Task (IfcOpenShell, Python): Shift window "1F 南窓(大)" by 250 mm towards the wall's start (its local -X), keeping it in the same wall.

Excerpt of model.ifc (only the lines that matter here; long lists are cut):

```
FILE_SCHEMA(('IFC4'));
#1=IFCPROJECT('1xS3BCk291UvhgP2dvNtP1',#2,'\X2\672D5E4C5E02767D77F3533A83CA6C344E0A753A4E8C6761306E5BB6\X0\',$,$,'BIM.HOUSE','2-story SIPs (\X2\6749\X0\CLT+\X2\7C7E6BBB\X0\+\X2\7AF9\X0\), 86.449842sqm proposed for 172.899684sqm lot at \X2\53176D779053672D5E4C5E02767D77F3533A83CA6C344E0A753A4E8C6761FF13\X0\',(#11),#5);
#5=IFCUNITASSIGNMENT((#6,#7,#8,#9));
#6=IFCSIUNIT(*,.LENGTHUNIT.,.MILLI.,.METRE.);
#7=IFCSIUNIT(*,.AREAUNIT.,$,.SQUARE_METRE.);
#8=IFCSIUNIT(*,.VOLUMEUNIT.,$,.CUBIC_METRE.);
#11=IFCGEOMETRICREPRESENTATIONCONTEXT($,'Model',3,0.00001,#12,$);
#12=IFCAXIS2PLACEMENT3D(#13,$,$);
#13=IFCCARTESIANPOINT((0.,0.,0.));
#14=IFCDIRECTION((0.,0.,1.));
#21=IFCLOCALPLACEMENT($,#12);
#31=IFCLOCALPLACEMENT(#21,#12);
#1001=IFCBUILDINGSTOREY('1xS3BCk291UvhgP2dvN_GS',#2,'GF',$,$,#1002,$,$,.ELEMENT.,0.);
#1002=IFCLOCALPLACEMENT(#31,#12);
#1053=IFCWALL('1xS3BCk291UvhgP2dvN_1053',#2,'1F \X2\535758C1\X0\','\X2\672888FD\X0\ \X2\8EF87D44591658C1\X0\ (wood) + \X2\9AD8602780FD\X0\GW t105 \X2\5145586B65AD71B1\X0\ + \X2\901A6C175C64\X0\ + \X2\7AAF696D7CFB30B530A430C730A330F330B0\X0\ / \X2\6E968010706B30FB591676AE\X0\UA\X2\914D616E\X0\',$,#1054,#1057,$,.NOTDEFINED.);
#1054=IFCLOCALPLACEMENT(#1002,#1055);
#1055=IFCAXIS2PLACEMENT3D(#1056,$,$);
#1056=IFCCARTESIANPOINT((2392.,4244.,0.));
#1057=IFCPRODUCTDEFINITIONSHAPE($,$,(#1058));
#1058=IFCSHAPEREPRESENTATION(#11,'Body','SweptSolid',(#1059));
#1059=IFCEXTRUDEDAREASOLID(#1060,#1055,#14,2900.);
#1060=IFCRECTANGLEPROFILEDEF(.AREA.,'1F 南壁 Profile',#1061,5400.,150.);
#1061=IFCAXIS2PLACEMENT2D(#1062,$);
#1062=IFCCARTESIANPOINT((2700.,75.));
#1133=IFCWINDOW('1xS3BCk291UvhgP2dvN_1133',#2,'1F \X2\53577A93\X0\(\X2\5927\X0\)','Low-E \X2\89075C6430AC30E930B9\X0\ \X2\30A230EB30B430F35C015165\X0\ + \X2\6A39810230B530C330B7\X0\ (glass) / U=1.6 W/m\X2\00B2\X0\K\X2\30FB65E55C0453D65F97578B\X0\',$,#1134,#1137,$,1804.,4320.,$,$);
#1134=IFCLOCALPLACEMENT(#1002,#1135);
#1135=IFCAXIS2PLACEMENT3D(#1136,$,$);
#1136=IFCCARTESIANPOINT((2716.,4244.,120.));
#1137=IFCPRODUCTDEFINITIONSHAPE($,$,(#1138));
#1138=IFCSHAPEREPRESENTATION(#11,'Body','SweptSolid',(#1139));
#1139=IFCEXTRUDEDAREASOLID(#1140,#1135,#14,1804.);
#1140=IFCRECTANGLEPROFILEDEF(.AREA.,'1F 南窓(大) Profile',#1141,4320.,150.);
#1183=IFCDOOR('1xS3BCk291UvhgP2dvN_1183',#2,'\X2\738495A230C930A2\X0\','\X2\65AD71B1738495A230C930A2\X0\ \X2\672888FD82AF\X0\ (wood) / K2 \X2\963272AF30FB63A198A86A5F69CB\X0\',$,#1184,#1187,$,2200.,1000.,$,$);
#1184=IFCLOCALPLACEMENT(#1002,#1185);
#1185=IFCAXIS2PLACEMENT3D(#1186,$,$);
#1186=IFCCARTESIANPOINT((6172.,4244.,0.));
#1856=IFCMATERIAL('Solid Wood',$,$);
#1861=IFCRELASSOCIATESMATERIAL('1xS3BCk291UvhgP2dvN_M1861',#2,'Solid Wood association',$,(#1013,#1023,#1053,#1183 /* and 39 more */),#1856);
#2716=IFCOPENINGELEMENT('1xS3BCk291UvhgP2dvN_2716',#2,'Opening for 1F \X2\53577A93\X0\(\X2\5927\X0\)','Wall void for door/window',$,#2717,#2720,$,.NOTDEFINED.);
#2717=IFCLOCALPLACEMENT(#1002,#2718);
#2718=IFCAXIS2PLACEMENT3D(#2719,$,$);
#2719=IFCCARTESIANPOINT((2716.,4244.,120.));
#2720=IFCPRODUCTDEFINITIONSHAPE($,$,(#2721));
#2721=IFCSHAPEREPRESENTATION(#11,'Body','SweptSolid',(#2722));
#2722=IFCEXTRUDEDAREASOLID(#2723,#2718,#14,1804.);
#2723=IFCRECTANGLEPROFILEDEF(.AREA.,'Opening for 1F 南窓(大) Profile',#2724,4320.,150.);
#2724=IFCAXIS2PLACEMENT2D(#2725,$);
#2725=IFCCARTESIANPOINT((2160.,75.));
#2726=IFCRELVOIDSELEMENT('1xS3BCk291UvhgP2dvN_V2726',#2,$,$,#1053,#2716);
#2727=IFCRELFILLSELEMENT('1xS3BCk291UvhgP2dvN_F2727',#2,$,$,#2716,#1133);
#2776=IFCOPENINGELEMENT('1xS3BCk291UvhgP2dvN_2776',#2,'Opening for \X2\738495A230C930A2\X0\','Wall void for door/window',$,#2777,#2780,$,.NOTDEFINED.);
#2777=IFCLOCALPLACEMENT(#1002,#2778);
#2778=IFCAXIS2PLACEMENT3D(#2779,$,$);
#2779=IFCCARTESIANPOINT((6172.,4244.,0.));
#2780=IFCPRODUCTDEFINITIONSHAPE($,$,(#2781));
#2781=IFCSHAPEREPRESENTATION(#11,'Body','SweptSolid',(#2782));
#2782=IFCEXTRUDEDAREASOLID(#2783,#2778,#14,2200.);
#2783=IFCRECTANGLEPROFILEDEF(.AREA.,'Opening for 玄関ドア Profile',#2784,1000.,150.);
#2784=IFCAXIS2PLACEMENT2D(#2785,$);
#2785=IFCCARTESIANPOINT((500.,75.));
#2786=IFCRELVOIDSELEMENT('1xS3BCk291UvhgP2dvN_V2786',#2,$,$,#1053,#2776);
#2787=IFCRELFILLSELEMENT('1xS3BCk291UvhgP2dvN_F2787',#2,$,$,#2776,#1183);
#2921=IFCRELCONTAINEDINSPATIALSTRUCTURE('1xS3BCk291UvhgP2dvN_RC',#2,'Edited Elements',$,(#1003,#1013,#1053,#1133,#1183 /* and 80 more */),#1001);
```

```python
import ifcopenshell
import ifcopenshell.api.geometry
import ifcopenshell.util.placement

model = ifcopenshell.open("model.ifc")

window = model.by_guid("1xS3BCk291UvhgP2dvN_1133")
opening = window.FillsVoids[0].RelatingOpeningElement
wall = opening.VoidsElements[0].RelatingBuildingElement

wall_matrix = ifcopenshell.util.placement.get_local_placement(wall.ObjectPlacement)
shift = wall_matrix[:3, 0] * -250.0
before = ifcopenshell.util.placement.get_local_placement(window.ObjectPlacement)[:3, 3].copy()

# The window is not placed relative to its opening, so move both.
for product in (opening, window):
    matrix = ifcopenshell.util.placement.get_local_placement(product.ObjectPlacement)
    matrix[:3, 3] += shift
    ifcopenshell.api.geometry.edit_object_placement(model, product=product, matrix=matrix, is_si=False)

after = ifcopenshell.util.placement.get_local_placement(window.ObjectPlacement)[:3, 3]
print("window moved by", (after - before).round(3) + 0.0)

model.write("model_v2.ifc")
```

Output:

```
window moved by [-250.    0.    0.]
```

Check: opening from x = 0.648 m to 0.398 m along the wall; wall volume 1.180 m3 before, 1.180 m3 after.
